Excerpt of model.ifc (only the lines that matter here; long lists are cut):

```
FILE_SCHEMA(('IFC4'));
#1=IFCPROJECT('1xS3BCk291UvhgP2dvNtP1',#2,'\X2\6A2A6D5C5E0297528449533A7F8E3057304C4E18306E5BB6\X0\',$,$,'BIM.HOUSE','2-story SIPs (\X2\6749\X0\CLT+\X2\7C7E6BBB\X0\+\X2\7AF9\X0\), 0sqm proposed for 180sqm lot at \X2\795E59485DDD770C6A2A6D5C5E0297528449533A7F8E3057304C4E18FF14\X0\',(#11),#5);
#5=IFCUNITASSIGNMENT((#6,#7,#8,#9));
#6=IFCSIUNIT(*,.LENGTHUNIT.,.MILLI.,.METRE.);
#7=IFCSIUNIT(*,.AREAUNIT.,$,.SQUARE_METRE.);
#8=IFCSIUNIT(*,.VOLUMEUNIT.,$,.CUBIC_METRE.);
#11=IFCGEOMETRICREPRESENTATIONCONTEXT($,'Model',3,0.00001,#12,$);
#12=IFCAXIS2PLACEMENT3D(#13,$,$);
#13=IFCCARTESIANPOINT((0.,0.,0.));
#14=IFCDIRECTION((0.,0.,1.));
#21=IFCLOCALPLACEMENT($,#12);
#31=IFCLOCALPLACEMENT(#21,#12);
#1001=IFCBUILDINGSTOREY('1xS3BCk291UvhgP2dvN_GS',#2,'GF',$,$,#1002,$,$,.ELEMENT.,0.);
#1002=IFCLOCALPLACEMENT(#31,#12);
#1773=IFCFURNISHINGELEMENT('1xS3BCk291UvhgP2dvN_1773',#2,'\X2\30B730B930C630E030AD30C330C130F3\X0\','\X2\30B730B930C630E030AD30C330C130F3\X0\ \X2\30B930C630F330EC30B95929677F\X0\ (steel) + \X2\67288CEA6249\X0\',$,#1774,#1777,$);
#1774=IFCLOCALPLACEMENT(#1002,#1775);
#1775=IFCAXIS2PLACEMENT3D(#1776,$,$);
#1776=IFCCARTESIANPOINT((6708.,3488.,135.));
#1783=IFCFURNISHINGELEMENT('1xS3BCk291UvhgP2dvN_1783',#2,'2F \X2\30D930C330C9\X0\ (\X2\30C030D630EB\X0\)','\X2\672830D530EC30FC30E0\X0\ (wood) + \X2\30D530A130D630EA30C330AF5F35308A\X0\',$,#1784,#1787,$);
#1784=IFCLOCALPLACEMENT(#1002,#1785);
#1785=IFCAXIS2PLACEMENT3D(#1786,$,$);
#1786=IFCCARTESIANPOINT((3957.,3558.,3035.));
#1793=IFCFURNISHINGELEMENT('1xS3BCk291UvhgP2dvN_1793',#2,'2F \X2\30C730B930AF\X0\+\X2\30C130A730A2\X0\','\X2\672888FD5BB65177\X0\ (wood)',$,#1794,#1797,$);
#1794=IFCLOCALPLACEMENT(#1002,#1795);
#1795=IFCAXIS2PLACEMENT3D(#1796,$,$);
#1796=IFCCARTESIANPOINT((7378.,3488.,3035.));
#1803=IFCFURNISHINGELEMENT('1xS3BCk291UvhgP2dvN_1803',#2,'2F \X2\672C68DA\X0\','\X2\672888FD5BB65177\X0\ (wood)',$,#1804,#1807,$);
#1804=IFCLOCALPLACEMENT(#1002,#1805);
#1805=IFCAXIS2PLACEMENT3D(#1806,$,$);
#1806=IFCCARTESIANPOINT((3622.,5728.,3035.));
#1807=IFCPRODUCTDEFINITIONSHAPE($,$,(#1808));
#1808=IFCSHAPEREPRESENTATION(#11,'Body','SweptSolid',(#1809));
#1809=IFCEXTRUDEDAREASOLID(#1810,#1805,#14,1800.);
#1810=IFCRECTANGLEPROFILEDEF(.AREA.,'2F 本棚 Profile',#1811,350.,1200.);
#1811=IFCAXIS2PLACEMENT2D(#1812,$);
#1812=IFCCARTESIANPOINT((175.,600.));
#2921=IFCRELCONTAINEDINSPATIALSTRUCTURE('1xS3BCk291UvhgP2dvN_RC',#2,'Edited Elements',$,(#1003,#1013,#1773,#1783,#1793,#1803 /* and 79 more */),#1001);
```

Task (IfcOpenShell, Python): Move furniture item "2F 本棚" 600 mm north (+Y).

```python
import ifcopenshell
import ifcopenshell.api.geometry
import ifcopenshell.util.placement
import ifcopenshell.util.unit

model = ifcopenshell.open("model.ifc")
unit_scale = ifcopenshell.util.unit.calculate_unit_scale(model)

item = model.by_guid("1xS3BCk291UvhgP2dvN_1803")
matrix = ifcopenshell.util.placement.get_local_placement(item.ObjectPlacement)
matrix[1, 3] += 0.6 / unit_scale
ifcopenshell.api.geometry.edit_object_placement(model, product=item, matrix=matrix, is_si=False)

print(ifcopenshell.util.placement.get_local_placement(item.ObjectPlacement).round(3) + 0.0)

model.write("model_edited.ifc")
```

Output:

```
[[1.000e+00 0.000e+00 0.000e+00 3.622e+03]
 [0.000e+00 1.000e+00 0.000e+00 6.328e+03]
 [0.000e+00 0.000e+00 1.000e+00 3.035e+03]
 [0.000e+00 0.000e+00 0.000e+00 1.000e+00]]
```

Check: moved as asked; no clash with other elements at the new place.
